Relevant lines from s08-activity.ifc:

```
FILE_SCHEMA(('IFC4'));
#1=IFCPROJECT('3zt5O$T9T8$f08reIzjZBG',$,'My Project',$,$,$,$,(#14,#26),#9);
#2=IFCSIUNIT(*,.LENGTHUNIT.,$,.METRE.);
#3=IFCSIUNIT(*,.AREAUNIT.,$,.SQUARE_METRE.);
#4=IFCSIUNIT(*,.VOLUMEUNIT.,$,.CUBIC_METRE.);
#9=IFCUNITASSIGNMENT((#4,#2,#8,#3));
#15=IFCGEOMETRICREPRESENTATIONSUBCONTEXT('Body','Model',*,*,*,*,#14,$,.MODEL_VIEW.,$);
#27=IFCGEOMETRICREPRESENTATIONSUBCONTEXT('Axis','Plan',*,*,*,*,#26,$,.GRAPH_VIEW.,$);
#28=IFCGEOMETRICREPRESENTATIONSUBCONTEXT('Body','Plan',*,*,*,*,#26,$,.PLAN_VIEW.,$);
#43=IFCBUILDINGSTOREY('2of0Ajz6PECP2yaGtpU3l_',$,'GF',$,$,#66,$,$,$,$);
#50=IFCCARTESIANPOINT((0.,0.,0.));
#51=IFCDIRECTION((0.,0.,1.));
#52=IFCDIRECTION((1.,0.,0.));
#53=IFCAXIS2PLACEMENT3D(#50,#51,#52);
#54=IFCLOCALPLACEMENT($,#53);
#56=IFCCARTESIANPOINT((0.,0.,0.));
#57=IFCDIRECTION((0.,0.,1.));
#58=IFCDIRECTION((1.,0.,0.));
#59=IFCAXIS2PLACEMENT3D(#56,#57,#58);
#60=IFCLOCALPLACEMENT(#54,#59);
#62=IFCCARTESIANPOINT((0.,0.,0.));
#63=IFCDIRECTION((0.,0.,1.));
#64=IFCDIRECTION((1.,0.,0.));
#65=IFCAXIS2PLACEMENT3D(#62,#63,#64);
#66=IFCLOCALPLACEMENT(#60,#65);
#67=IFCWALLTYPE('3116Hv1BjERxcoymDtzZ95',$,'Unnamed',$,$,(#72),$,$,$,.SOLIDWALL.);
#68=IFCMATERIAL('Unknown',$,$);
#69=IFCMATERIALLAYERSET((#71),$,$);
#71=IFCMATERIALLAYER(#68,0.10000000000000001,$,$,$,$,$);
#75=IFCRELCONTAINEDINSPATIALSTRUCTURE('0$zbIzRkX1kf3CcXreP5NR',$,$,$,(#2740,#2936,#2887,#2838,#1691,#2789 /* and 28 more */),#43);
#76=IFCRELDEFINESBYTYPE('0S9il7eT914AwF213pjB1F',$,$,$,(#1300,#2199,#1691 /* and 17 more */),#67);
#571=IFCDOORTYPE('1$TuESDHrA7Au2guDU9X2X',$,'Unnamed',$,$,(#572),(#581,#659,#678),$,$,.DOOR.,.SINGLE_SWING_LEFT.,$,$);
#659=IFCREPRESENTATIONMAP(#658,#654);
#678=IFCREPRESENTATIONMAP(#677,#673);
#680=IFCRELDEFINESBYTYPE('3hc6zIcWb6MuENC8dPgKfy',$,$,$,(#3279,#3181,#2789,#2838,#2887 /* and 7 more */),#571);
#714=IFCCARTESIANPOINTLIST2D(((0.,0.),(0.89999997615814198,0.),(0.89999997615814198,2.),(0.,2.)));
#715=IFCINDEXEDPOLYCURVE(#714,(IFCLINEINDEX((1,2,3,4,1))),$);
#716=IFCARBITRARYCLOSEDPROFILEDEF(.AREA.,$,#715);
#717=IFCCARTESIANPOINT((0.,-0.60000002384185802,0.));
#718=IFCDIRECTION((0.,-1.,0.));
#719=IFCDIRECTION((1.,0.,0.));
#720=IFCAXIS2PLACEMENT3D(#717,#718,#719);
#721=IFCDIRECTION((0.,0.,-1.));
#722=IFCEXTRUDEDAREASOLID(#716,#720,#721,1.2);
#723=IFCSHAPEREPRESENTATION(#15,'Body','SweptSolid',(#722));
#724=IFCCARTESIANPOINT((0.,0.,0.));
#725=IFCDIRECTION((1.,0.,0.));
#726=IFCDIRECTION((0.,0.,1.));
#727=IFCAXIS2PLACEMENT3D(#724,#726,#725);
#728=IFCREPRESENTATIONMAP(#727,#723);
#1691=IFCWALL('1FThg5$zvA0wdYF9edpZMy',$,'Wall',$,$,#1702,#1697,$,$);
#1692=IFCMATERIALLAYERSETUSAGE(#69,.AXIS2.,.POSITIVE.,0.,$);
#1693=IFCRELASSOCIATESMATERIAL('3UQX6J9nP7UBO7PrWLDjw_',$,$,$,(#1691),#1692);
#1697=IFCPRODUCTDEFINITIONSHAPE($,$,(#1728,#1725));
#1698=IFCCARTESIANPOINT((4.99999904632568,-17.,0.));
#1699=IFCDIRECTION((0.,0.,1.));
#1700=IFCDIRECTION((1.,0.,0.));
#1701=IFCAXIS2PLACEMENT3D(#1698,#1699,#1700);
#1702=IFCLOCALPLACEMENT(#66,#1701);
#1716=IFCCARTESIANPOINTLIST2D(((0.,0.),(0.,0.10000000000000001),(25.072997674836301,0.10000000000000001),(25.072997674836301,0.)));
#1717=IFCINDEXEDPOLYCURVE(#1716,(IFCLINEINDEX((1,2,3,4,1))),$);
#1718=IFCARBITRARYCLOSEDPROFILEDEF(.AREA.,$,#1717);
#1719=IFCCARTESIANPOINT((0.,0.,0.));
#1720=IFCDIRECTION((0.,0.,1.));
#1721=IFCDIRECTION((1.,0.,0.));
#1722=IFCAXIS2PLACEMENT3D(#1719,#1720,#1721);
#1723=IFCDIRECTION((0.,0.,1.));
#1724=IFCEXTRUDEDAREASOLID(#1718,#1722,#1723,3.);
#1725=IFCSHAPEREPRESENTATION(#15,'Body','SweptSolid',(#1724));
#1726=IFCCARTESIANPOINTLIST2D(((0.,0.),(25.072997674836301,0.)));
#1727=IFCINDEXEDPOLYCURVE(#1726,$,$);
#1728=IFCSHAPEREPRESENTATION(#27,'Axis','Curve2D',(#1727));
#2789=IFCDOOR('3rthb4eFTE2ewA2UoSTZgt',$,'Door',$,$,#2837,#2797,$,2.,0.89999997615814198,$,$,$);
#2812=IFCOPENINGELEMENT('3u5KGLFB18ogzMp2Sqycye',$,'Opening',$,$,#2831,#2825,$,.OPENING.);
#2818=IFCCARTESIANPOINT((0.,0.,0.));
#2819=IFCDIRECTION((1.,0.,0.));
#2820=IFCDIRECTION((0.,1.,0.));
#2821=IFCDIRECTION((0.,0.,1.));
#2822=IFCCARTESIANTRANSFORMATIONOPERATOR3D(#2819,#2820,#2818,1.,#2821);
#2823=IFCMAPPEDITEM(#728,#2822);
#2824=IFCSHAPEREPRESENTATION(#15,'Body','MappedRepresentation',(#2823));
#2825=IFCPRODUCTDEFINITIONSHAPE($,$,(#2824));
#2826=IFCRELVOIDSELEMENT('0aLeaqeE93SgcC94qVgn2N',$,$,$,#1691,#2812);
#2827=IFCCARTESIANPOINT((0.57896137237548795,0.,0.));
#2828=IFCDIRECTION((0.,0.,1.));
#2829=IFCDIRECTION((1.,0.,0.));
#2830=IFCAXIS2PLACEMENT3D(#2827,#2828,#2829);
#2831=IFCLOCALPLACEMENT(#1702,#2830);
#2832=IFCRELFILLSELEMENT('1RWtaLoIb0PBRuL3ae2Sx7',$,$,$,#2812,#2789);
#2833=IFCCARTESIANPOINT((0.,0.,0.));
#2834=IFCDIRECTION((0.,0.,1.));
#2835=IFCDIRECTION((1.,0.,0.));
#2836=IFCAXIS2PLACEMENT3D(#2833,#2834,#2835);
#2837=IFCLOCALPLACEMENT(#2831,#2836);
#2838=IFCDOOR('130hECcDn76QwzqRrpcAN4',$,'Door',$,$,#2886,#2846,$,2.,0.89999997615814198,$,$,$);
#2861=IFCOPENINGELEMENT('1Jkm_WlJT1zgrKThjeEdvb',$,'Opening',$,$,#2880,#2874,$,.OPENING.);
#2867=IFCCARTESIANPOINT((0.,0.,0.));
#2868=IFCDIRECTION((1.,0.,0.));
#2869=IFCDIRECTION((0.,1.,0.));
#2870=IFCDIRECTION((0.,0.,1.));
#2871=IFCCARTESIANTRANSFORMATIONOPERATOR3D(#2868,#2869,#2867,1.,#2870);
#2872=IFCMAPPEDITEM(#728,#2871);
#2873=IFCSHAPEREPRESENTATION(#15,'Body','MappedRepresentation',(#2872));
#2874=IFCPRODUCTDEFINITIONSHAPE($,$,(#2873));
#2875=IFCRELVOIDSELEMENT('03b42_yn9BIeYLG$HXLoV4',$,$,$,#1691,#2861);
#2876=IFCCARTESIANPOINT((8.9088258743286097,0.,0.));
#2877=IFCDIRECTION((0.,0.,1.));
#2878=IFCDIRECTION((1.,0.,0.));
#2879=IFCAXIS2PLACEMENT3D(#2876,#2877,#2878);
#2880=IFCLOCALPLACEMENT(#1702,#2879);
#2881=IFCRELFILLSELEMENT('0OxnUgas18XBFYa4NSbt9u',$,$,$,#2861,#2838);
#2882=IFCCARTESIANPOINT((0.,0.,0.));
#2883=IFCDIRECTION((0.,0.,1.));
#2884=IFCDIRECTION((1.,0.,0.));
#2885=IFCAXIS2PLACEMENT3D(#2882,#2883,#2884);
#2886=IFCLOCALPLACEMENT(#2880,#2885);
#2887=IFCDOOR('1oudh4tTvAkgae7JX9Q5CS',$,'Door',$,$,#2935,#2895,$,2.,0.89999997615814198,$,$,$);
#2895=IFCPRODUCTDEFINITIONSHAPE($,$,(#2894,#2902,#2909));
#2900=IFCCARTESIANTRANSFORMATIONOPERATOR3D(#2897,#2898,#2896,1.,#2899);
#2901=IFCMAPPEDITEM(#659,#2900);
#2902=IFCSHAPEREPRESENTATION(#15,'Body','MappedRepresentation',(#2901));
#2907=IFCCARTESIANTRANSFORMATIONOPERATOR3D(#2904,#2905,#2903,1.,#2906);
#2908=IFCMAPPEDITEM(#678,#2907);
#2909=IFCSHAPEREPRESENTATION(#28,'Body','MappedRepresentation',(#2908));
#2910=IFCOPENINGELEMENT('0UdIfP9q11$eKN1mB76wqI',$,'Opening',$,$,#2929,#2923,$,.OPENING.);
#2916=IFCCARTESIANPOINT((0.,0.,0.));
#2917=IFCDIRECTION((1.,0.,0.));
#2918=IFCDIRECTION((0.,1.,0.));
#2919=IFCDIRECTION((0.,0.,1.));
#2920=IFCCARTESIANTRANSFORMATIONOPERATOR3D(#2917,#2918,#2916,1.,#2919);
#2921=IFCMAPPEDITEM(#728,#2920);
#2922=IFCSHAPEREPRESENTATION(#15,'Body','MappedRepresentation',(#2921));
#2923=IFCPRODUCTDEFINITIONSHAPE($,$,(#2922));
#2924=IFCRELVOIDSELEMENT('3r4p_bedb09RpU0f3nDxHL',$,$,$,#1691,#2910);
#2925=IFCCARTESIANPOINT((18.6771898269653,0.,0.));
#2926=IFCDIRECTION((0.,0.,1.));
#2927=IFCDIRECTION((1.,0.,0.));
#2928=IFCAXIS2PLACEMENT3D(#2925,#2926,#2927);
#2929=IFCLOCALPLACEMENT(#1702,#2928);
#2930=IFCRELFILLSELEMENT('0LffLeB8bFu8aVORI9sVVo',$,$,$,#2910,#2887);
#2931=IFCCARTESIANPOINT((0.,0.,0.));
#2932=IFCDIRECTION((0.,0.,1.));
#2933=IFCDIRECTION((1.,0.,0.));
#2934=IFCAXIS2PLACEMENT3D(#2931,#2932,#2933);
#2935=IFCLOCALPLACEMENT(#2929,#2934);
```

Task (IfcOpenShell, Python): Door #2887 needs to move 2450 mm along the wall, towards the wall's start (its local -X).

```python
import ifcopenshell
import ifcopenshell.api.geometry
import ifcopenshell.util.placement
import ifcopenshell.util.unit

model = ifcopenshell.open("s08-activity.ifc")
unit_scale = ifcopenshell.util.unit.calculate_unit_scale(model)

door = model.by_id(2887)
opening = door.FillsVoids[0].RelatingOpeningElement
wall = opening.VoidsElements[0].RelatingBuildingElement

wall_matrix = ifcopenshell.util.placement.get_local_placement(wall.ObjectPlacement)
shift = wall_matrix[:3, 0] * -2.45 / unit_scale
before = ifcopenshell.util.placement.get_local_placement(door.ObjectPlacement)[:3, 3].copy()

# The door is placed relative to its opening, so it follows when the opening moves.
matrix = ifcopenshell.util.placement.get_local_placement(opening.ObjectPlacement)
matrix[:3, 3] += shift
ifcopenshell.api.geometry.edit_object_placement(
    model, product=opening, matrix=matrix, is_si=False, should_transform_children=True
)

after = ifcopenshell.util.placement.get_local_placement(door.ObjectPlacement)[:3, 3]
print("door moved by", (after - before).round(3) + 0.0)

model.write("s08-activity_v2.ifc")
```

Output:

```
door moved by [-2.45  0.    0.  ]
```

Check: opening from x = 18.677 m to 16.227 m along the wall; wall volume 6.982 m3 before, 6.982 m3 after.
